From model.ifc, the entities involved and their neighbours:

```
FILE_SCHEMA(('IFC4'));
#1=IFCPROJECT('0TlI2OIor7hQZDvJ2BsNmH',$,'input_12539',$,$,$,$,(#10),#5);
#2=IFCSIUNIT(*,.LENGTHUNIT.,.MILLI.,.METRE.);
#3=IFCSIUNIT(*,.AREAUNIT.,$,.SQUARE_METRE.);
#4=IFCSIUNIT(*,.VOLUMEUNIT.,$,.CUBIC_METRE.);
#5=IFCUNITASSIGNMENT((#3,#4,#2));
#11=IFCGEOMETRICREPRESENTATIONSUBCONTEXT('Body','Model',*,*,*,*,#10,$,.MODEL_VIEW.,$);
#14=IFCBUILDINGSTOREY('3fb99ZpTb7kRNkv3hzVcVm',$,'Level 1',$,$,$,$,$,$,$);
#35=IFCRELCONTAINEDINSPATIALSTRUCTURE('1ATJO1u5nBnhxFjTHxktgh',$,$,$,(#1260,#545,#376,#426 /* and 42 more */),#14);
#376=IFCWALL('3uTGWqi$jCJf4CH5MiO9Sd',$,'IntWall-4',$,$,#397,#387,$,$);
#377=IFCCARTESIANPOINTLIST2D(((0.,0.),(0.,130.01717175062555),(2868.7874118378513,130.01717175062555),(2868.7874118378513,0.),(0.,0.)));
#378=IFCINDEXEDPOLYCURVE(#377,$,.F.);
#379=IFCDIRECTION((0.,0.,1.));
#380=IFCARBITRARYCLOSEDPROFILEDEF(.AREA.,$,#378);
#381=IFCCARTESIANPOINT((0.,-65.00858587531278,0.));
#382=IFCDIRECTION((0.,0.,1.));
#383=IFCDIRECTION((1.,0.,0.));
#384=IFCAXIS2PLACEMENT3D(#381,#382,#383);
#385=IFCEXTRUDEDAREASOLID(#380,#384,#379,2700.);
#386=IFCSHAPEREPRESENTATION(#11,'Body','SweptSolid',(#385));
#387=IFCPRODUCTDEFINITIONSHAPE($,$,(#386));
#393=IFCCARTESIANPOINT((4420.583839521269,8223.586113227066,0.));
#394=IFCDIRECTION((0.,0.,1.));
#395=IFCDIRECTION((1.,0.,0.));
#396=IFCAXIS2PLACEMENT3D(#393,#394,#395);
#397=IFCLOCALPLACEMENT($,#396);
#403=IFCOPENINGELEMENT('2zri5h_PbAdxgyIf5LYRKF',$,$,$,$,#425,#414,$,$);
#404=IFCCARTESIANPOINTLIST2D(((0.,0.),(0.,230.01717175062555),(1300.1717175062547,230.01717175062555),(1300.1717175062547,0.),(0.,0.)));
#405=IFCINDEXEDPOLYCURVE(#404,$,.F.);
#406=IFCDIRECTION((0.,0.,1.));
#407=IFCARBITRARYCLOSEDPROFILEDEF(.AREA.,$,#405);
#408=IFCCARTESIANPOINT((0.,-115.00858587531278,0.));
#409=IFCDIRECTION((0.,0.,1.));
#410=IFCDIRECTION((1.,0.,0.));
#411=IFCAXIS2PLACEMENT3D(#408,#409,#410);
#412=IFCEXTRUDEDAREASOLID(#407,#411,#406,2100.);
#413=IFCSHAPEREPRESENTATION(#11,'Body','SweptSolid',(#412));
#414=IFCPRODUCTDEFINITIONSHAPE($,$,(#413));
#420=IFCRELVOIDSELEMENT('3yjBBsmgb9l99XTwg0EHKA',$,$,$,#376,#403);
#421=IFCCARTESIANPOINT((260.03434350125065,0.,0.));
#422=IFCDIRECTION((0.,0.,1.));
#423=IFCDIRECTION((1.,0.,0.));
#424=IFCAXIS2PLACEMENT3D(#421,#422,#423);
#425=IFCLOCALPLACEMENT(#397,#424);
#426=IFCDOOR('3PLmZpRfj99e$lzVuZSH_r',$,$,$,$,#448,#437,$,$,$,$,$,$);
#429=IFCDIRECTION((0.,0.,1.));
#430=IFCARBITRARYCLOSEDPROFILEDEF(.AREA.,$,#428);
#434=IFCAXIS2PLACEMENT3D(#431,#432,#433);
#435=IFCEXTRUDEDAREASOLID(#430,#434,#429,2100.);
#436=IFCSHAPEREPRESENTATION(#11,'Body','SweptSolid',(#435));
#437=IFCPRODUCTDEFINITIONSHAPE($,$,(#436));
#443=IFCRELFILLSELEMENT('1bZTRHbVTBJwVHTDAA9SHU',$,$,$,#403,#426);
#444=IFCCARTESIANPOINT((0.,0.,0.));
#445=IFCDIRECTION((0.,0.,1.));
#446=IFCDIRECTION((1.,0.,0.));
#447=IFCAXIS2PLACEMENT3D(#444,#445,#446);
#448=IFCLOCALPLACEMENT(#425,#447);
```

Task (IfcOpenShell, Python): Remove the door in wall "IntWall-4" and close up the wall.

```python
import ifcopenshell
import ifcopenshell.api.feature
import ifcopenshell.api.root
import ifcopenshell.geom
import ifcopenshell.util.shape

model = ifcopenshell.open("model.ifc")
settings = ifcopenshell.geom.settings()


def volume(element):
    """Net volume in cubic metres, openings subtracted."""
    shape = ifcopenshell.geom.create_shape(settings, element)
    return ifcopenshell.util.shape.get_volume(shape.geometry)


door = model.by_guid("3PLmZpRfj99e$lzVuZSH_r")
opening = door.FillsVoids[0].RelatingOpeningElement
wall = opening.VoidsElements[0].RelatingBuildingElement
before = volume(wall)

ifcopenshell.api.root.remove_product(model, product=door)
ifcopenshell.api.feature.remove_feature(model, feature=opening)

after = volume(wall)

print(f"wall volume {before:.3f} -> {after:.3f} m3")

model.write("model-out.ifc")
```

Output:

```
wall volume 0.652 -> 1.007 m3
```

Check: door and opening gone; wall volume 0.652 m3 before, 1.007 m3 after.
